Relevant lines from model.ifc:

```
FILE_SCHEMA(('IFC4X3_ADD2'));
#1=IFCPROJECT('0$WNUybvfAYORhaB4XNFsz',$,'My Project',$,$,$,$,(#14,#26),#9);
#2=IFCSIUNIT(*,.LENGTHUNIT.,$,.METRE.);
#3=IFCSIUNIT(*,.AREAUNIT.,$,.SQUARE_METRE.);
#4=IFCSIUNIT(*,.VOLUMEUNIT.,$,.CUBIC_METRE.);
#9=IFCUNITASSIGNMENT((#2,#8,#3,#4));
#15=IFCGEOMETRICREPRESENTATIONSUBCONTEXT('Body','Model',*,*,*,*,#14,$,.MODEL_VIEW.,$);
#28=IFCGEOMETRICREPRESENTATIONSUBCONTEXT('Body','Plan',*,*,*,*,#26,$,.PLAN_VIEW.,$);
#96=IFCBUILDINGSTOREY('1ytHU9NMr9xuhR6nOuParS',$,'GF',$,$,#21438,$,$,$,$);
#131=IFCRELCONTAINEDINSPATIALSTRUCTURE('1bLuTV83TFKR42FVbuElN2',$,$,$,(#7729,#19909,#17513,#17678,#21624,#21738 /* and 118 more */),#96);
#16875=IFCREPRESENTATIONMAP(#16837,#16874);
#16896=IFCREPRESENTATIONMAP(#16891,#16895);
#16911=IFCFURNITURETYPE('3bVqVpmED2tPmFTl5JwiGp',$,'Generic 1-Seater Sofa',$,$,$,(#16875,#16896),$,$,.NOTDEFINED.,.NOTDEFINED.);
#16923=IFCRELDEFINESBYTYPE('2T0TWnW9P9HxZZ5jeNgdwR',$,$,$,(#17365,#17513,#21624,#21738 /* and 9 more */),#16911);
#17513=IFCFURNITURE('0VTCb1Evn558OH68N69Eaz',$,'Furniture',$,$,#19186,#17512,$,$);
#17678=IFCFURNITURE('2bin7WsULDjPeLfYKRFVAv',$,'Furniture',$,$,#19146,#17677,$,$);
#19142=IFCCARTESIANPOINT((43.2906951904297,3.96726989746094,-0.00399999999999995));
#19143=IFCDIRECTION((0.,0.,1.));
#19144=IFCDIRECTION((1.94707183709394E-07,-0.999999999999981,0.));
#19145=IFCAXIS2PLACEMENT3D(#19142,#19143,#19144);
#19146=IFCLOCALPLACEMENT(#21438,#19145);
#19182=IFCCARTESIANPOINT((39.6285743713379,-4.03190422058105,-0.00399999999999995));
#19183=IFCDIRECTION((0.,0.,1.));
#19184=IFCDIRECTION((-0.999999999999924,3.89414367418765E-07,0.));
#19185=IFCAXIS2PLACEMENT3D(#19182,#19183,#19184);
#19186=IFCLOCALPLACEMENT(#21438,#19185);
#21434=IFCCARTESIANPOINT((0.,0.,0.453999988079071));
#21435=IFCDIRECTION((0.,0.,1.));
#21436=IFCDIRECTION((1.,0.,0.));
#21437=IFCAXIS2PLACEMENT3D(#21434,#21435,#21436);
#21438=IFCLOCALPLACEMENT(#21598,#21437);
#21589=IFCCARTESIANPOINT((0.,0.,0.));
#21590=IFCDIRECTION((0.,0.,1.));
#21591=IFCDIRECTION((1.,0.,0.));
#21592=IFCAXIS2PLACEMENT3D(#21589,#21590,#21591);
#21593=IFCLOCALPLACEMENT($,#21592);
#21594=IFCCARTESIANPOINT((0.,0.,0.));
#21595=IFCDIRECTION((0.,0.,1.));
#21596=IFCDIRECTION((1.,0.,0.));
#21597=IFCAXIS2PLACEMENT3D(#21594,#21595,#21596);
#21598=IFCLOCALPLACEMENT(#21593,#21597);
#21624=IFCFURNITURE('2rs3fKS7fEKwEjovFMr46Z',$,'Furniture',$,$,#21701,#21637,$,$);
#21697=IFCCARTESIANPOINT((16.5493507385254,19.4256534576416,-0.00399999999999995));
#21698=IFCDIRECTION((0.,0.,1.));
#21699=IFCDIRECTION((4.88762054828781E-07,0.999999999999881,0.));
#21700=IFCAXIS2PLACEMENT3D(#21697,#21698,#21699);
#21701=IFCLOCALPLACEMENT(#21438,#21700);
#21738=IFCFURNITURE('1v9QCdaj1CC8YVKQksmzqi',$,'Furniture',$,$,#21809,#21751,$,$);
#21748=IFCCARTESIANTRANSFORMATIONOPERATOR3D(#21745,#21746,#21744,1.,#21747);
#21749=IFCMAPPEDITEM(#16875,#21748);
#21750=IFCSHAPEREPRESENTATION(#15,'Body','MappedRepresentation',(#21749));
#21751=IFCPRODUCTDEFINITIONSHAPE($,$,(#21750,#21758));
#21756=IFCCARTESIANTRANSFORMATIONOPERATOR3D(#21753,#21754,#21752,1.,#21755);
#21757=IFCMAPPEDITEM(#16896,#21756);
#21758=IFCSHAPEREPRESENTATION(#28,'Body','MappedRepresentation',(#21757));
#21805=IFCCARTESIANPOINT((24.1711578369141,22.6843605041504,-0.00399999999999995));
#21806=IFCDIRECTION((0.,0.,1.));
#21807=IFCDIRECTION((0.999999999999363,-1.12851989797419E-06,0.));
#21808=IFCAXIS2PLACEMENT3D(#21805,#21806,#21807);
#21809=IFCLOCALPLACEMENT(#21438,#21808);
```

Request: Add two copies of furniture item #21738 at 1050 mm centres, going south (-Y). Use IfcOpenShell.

```python
import numpy as np
import ifcopenshell
import ifcopenshell.api.geometry
import ifcopenshell.api.root
import ifcopenshell.util.element
import ifcopenshell.util.placement

model = ifcopenshell.open("model.ifc")

source = model.by_id(21738)
base = ifcopenshell.util.placement.get_local_placement(source.ObjectPlacement)
step = np.array([0.0, -1.0, 0.0]) * 1.05

for i in range(1, 3):
    copy = ifcopenshell.api.root.copy_class(model, product=source)
    copy.Representation = ifcopenshell.util.element.copy_deep(
        model, source.Representation, exclude=["IfcGeometricRepresentationContext", "IfcRepresentationMap"]
    )
    matrix = base.copy()
    matrix[:3, 3] += i * step
    print("added at", matrix[:3, 3].round(3) + 0.0)
    ifcopenshell.api.geometry.edit_object_placement(model, product=copy, matrix=matrix, is_si=False)

model.write("model_edited.ifc")
```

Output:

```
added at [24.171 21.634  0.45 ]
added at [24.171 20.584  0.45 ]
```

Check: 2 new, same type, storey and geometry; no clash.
